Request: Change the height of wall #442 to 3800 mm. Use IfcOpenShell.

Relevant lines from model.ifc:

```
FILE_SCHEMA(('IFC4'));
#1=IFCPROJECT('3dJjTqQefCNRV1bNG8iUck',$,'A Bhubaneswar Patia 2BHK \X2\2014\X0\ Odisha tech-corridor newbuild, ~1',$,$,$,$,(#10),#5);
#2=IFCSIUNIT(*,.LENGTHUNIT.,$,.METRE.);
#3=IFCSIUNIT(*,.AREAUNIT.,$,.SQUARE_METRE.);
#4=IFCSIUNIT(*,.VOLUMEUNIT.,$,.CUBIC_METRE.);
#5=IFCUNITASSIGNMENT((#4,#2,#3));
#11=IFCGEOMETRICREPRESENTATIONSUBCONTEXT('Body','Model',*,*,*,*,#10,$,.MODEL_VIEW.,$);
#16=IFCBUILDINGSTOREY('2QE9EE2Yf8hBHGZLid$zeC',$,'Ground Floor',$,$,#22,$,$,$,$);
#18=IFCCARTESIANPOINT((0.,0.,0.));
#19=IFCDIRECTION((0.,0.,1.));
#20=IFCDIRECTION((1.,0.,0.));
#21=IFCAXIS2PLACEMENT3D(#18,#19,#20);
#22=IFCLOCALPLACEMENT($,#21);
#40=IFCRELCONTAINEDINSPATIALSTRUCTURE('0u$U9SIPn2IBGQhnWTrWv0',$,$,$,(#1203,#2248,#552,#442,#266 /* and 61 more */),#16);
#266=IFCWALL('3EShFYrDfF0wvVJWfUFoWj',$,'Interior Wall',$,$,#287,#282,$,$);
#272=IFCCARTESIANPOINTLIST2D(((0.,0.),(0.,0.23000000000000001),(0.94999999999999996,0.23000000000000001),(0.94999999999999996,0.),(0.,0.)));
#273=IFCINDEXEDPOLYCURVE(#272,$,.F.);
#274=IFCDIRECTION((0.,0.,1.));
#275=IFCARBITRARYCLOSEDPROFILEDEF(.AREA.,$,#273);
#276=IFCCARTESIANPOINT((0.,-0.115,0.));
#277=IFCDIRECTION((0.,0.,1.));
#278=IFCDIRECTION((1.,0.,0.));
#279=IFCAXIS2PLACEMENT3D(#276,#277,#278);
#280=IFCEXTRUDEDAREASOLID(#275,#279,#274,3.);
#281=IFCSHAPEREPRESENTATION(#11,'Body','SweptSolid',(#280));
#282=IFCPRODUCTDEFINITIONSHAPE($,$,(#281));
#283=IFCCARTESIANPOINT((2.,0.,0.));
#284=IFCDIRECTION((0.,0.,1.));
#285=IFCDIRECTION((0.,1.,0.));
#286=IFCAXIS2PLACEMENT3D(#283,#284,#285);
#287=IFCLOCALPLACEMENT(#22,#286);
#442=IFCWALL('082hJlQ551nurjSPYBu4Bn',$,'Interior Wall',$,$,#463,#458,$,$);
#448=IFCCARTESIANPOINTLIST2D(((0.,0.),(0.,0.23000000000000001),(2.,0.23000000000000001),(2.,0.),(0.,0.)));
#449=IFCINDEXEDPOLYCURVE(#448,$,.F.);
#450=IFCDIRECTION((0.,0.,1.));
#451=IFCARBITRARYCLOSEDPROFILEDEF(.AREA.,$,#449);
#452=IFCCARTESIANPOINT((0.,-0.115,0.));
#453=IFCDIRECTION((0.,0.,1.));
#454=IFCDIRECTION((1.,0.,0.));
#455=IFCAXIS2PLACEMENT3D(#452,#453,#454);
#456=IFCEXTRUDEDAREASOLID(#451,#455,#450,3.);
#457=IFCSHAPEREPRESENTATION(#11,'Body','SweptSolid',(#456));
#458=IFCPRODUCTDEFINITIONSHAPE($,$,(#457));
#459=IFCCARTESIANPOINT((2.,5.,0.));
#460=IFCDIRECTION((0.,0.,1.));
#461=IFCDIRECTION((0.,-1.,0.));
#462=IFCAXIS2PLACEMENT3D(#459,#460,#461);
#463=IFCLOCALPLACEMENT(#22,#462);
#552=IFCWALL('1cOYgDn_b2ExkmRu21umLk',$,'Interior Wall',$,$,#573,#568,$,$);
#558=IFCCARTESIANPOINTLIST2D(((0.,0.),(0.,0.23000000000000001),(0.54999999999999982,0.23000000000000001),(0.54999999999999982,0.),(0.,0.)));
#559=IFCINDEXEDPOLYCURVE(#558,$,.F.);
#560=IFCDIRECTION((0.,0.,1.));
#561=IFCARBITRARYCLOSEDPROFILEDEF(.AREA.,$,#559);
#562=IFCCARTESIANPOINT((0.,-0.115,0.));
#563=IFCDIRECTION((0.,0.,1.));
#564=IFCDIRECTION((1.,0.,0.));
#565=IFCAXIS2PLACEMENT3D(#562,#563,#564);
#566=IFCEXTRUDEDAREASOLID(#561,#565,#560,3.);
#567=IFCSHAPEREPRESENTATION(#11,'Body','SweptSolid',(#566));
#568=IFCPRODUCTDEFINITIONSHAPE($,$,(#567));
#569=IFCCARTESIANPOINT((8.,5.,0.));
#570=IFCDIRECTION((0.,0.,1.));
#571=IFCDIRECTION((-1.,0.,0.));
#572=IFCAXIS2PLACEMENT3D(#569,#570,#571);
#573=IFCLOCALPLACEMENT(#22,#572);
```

```python
import ifcopenshell
import ifcopenshell.geom
import ifcopenshell.util.representation
import ifcopenshell.util.shape
import ifcopenshell.util.unit

model = ifcopenshell.open("model.ifc")
unit_scale = ifcopenshell.util.unit.calculate_unit_scale(model)
settings = ifcopenshell.geom.settings()


def volume(element):
    """Net volume in cubic metres, openings subtracted."""
    shape = ifcopenshell.geom.create_shape(settings, element)
    return ifcopenshell.util.shape.get_volume(shape.geometry)


wall = model.by_guid("082hJlQ551nurjSPYBu4Bn")
before = volume(wall)

body = ifcopenshell.util.representation.get_representation(wall, "Model", "Body")
solid = body.Items[0]
old_height = solid.Depth
solid.Depth = 3.8 / unit_scale
after = volume(wall)

print(f"height {old_height:g} -> {solid.Depth:g}, volume {before:.3f} -> {after:.3f} m3")

model.write("model_edited.ifc")
```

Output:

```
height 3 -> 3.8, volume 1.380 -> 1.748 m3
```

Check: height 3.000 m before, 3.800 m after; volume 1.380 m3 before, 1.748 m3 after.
